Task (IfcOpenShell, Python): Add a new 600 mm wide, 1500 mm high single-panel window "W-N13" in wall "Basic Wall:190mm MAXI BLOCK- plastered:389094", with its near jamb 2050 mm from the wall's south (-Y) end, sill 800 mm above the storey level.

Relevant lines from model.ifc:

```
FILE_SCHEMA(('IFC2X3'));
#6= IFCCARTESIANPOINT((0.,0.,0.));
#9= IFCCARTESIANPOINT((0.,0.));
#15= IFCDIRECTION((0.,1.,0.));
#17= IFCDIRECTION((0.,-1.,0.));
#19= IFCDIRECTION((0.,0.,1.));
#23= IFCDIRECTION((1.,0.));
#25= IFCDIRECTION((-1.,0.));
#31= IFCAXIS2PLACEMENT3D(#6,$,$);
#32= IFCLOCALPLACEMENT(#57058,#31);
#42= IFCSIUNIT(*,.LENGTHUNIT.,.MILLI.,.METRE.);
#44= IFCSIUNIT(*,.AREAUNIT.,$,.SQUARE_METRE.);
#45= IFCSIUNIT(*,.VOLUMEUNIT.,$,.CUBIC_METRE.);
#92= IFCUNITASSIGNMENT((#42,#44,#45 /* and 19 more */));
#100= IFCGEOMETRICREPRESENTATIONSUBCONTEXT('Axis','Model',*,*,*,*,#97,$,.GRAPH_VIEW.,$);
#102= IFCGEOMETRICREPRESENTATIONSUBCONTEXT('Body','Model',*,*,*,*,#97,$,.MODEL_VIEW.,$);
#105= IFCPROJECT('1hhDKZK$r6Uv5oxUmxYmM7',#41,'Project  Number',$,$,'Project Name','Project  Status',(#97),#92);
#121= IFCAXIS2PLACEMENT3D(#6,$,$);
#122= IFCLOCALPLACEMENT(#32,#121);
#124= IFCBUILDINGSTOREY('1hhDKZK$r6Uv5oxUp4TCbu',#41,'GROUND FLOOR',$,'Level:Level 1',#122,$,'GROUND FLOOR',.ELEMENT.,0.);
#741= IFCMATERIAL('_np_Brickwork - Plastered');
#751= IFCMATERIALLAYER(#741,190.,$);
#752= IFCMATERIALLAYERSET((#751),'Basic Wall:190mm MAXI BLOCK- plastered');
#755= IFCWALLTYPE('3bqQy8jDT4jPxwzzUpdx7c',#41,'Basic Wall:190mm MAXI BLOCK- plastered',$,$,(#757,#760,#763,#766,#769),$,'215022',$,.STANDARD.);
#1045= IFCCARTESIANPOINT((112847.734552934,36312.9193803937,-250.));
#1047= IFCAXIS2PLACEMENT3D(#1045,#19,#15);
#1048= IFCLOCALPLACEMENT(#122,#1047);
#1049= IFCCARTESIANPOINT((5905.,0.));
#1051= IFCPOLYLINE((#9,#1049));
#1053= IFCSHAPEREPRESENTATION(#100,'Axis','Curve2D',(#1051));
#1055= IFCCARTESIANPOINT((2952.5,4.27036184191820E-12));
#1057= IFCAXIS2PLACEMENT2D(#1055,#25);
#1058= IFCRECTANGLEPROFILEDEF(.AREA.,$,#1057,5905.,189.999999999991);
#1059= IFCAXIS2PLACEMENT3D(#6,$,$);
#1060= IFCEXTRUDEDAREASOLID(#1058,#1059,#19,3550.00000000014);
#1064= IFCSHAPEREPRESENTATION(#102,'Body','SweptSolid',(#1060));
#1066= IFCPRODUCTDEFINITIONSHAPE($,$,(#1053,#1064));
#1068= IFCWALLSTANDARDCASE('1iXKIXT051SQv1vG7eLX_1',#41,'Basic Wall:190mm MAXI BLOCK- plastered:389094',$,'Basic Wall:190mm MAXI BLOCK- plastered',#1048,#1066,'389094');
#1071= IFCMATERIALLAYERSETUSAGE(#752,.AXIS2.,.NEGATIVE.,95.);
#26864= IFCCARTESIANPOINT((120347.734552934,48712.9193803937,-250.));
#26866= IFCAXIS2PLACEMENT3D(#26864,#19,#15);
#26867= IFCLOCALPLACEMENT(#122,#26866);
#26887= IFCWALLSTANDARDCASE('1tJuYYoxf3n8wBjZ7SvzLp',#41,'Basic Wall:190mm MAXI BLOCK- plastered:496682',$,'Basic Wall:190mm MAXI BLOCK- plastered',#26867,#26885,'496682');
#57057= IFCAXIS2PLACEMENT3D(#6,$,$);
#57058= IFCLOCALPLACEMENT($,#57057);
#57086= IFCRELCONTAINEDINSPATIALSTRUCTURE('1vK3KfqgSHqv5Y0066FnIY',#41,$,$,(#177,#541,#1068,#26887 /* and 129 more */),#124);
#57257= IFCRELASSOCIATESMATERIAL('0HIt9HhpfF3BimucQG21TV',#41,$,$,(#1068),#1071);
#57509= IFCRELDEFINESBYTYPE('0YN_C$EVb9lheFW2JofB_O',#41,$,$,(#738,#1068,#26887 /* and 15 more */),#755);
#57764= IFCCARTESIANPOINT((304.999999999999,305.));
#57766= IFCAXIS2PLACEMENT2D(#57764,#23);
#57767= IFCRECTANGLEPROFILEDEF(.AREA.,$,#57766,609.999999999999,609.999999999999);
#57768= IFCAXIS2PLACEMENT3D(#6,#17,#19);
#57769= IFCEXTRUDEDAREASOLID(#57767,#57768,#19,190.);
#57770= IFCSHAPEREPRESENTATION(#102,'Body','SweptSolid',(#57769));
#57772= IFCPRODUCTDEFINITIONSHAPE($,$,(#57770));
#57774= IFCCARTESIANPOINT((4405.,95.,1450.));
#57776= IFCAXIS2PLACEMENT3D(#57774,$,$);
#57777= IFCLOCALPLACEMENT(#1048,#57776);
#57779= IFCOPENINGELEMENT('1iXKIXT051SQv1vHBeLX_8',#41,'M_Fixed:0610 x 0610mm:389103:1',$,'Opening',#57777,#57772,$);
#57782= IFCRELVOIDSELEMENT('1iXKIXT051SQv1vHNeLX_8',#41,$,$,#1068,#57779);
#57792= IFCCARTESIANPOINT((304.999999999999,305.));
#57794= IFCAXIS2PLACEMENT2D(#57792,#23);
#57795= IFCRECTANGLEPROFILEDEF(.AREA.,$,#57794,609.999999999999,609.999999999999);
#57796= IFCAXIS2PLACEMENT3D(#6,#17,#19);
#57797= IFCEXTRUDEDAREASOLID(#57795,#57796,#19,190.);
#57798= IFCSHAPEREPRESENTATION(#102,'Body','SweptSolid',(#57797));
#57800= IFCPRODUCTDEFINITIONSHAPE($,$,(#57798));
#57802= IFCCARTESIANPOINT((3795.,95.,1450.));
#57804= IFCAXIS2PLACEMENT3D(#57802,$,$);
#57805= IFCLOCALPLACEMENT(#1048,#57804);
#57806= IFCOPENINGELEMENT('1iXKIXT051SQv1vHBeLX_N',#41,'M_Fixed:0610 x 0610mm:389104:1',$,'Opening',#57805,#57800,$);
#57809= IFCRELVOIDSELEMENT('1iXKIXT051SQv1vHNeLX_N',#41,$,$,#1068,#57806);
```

```python
import numpy as np
import ifcopenshell
import ifcopenshell.api.feature
import ifcopenshell.api.geometry
import ifcopenshell.api.root
import ifcopenshell.api.spatial
import ifcopenshell.api.type
import ifcopenshell.geom
import ifcopenshell.util.element
import ifcopenshell.util.placement
import ifcopenshell.util.representation
import ifcopenshell.util.shape
import ifcopenshell.util.unit

model = ifcopenshell.open("model.ifc")
unit_scale = ifcopenshell.util.unit.calculate_unit_scale(model)
settings = ifcopenshell.geom.settings()


def volume(element):
    """Net volume in cubic metres, openings subtracted."""
    shape = ifcopenshell.geom.create_shape(settings, element)
    return ifcopenshell.util.shape.get_volume(shape.geometry)


wall = model.by_guid("1iXKIXT051SQv1vG7eLX_1")
storey = ifcopenshell.util.element.get_container(wall, ifc_class="IfcBuildingStorey")
context = ifcopenshell.util.representation.get_context(model, "Model", "Body", "MODEL_VIEW")
before = volume(wall)

width, height, from_end, sill = 0.6, 1.5, 2.05, 0.8  # metres

# The wall runs along its own X axis, and the end named is its -X end.
wall_shape = ifcopenshell.geom.create_shape(settings, wall)
x, y, z = ifcopenshell.util.shape.get_vertices(wall_shape.geometry).T
start = x.min() + from_end
face, thickness = float(y.min()), float(y.max() - y.min())
wall_matrix = ifcopenshell.util.placement.get_local_placement(wall.ObjectPlacement)
level = ifcopenshell.util.placement.get_local_placement(storey.ObjectPlacement)[2, 3]


def in_wall(x, y):
    """Placement at x, y metres in the wall's axes, at sill height."""
    matrix = wall_matrix.copy()
    matrix[:, 3] = wall_matrix @ np.array([x / unit_scale, y / unit_scale, 0.0, 1.0])
    matrix[2, 3] = level + sill / unit_scale
    return matrix


# Opening: a box that overshoots both wall faces by 50 mm.
opening = ifcopenshell.api.root.create_entity(model, ifc_class="IfcOpeningElement")
box = ifcopenshell.api.geometry.add_wall_representation(
    model, context=context, length=width, height=height, thickness=thickness + 0.1
)
ifcopenshell.api.geometry.assign_representation(model, product=opening, representation=box)
ifcopenshell.api.geometry.edit_object_placement(model, product=opening, matrix=in_wall(start, face - 0.05), is_si=False)
ifcopenshell.api.feature.add_feature(model, feature=opening, element=wall)

window = ifcopenshell.api.root.create_entity(model, ifc_class="IfcWindow", name="W-N13")
window.OverallWidth, window.OverallHeight = width / unit_scale, height / unit_scale
body = ifcopenshell.api.geometry.add_window_representation(
    model,
    context=context,
    overall_width=window.OverallWidth,
    overall_height=window.OverallHeight,
    partition_type="SINGLE_PANEL",
)
ifcopenshell.api.geometry.assign_representation(model, product=window, representation=body)
ifcopenshell.api.spatial.assign_container(model, products=[window], relating_structure=storey)
fills = ifcopenshell.api.feature.add_filling(model, opening=opening, element=window)
fills.OwnerHistory = window.OwnerHistory  # required in IFC2X3

# IFC2X3 keeps the operation on the window style.
style = ifcopenshell.api.root.create_entity(model, ifc_class="IfcWindowStyle", name="W-N13")
style.OperationType, style.ConstructionType = "SINGLE_PANEL", "NOTDEFINED"
style.ParameterTakesPrecedence = style.Sizeable = False
ifcopenshell.api.type.assign_type(model, related_objects=[window], relating_type=style)

# Centre the window in the wall's thickness.
ifcopenshell.api.geometry.edit_object_placement(model, product=window, matrix=in_wall(start, face), is_si=False)
window_shape = ifcopenshell.geom.create_shape(settings, window)
depth = ifcopenshell.util.shape.get_vertices(window_shape.geometry)[:, 1]
offset = face + thickness / 2 - (depth.min() + depth.max()) / 2
ifcopenshell.api.geometry.edit_object_placement(model, product=window, matrix=in_wall(start, offset), is_si=False)

after = volume(wall)

print(f"wall volume {before:.3f} -> {after:.3f} m3")

model.write("model_rev.ifc")
```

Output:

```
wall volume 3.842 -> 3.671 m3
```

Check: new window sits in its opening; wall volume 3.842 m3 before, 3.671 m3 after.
